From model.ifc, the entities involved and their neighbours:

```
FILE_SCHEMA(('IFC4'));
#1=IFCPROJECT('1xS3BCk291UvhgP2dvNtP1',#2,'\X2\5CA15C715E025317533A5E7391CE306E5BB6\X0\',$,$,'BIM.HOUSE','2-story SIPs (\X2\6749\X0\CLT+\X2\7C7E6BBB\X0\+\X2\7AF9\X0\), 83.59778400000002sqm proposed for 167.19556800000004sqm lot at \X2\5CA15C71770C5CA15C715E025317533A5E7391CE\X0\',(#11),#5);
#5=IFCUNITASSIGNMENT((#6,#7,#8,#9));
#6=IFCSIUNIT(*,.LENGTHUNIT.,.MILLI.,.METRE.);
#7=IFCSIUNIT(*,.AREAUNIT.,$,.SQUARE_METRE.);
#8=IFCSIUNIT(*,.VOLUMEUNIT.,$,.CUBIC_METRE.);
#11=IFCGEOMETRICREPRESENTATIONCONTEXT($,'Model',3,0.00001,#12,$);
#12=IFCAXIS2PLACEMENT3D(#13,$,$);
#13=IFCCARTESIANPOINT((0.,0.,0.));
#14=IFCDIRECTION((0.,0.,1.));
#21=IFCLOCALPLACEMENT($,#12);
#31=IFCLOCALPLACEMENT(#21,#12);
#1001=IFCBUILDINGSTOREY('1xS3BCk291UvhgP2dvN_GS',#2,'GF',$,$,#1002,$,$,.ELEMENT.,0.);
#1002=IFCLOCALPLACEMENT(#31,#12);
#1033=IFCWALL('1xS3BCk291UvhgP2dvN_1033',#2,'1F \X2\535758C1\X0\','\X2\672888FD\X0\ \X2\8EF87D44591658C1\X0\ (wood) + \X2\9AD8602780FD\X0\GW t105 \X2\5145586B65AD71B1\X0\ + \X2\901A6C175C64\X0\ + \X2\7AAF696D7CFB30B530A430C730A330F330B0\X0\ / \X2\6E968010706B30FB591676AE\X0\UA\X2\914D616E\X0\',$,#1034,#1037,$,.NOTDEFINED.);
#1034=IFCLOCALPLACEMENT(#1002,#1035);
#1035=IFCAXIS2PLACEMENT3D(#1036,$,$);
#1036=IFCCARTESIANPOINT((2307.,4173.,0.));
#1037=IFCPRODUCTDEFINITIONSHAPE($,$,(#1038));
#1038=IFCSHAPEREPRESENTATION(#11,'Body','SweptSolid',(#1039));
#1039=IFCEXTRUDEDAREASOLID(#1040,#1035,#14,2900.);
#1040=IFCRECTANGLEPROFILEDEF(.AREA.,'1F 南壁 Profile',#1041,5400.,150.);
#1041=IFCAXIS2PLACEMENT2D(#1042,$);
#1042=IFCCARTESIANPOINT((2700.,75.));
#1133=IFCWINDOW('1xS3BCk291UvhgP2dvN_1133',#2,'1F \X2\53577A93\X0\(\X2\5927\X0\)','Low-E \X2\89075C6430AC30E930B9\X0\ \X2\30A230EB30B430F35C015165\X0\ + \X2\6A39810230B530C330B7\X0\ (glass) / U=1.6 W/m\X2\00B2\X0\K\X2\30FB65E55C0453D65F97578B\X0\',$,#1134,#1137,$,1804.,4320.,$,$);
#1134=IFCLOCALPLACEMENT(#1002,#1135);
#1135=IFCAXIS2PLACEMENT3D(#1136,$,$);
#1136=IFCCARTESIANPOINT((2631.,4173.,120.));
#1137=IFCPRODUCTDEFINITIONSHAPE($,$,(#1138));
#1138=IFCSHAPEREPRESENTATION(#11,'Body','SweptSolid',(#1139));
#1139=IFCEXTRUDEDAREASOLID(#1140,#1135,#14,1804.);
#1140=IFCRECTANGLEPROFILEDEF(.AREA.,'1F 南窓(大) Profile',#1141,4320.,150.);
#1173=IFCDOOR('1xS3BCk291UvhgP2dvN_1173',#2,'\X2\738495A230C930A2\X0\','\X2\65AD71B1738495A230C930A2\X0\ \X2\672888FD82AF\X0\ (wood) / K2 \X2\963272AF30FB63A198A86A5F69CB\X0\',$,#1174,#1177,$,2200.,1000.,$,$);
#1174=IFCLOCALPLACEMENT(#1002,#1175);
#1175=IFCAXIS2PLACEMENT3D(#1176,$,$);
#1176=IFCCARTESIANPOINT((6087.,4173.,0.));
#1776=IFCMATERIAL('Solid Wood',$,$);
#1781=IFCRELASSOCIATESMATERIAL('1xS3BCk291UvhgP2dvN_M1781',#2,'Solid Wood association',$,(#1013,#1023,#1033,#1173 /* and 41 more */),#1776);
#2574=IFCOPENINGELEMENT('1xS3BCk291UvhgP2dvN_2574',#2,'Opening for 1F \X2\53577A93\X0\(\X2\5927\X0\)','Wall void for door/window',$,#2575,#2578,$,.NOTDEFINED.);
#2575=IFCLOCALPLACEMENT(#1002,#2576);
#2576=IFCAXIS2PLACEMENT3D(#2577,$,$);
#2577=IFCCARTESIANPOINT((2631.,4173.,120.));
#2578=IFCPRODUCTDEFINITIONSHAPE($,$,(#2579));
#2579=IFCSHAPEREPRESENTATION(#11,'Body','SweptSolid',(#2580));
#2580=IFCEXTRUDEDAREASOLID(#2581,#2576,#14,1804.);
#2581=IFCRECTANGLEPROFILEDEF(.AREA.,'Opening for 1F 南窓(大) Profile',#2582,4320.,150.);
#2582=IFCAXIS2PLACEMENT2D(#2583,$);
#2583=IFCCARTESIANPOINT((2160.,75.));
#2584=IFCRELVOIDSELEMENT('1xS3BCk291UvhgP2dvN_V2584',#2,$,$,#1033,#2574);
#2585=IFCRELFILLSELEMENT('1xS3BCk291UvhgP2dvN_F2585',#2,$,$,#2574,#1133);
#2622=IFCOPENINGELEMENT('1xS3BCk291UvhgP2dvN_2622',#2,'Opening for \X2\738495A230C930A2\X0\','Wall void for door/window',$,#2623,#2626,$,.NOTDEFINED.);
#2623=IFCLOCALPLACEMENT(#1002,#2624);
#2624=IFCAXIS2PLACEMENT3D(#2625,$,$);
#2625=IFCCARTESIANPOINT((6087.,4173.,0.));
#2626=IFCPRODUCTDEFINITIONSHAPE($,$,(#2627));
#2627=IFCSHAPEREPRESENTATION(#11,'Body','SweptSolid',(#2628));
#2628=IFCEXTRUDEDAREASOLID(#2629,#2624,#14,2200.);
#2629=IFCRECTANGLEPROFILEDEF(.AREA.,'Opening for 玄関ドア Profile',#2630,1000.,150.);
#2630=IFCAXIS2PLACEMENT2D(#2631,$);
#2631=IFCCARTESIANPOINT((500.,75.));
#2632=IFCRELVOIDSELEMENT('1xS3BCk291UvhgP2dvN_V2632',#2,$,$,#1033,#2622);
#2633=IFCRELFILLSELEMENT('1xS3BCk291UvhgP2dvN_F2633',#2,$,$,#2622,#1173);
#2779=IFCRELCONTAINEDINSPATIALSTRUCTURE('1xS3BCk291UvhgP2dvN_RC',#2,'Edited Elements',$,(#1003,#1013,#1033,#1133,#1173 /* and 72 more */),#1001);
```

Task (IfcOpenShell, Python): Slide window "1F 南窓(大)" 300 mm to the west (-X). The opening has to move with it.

```python
import ifcopenshell
import ifcopenshell.api.geometry
import ifcopenshell.util.placement

model = ifcopenshell.open("model.ifc")

window = model.by_guid("1xS3BCk291UvhgP2dvN_1133")
opening = window.FillsVoids[0].RelatingOpeningElement
wall = opening.VoidsElements[0].RelatingBuildingElement

wall_matrix = ifcopenshell.util.placement.get_local_placement(wall.ObjectPlacement)
shift = wall_matrix[:3, 0] * -300.0
before = ifcopenshell.util.placement.get_local_placement(window.ObjectPlacement)[:3, 3].copy()

# The window is not placed relative to its opening, so move both.
for product in (opening, window):
    matrix = ifcopenshell.util.placement.get_local_placement(product.ObjectPlacement)
    matrix[:3, 3] += shift
    ifcopenshell.api.geometry.edit_object_placement(model, product=product, matrix=matrix, is_si=False)

after = ifcopenshell.util.placement.get_local_placement(window.ObjectPlacement)[:3, 3]
print("window moved by", (after - before).round(3) + 0.0)

model.write("model-out.ifc")
```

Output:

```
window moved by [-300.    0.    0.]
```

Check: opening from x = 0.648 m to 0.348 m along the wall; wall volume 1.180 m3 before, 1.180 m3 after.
